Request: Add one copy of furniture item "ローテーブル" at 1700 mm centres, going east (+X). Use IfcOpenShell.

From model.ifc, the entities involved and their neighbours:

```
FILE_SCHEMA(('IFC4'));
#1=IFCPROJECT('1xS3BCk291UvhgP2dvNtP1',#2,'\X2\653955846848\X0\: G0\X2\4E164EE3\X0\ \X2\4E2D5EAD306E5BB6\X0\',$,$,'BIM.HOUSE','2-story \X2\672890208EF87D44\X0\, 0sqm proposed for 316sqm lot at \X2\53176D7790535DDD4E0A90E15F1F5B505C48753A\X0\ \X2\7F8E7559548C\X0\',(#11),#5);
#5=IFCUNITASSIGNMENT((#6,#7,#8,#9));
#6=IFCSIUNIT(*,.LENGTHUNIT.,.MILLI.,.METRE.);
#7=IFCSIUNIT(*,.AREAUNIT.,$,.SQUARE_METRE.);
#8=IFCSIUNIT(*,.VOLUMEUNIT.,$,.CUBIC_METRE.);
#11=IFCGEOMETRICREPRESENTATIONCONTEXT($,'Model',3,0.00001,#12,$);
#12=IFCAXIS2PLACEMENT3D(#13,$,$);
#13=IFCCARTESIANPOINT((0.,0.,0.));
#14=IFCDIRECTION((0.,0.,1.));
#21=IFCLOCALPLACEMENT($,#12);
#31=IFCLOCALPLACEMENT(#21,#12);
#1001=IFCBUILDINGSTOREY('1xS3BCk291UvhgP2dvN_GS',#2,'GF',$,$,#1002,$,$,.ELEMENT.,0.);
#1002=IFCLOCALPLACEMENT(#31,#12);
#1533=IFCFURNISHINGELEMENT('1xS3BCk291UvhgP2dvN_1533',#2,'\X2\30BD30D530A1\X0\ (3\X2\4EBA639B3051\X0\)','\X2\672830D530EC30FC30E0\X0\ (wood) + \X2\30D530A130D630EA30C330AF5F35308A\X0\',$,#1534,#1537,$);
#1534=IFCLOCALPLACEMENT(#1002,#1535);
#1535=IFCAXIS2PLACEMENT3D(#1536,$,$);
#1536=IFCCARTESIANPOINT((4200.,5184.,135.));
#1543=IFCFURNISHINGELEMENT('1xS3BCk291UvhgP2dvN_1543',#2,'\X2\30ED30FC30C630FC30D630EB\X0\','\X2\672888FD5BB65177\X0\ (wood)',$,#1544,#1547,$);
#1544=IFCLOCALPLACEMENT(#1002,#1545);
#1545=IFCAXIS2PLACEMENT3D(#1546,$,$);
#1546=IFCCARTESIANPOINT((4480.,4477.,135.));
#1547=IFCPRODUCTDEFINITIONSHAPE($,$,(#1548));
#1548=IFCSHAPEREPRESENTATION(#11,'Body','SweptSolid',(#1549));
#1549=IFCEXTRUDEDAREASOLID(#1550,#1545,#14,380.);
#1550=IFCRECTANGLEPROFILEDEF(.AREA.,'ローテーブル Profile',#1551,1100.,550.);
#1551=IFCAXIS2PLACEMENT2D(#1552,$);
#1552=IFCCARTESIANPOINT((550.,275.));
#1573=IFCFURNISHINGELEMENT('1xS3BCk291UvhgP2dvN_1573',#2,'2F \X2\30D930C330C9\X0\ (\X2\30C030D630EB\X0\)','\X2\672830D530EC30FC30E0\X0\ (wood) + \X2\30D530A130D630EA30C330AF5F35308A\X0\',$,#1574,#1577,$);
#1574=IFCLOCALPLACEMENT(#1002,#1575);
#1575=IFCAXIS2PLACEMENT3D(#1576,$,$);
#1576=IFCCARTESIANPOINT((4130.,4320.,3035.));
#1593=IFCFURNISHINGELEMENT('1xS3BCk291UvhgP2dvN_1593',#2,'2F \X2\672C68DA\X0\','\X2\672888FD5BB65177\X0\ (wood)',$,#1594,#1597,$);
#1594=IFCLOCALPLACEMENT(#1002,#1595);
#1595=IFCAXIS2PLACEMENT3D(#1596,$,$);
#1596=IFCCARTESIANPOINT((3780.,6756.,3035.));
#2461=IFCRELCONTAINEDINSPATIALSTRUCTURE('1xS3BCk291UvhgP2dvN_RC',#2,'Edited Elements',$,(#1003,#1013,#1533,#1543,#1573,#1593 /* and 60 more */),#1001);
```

```python
import numpy as np
import ifcopenshell
import ifcopenshell.api.geometry
import ifcopenshell.api.root
import ifcopenshell.util.element
import ifcopenshell.util.placement

model = ifcopenshell.open("model.ifc")


def reuse_history(source, copy):
    """copy_class also copies each property set's owner history, people and application; keep the originals."""
    for rel in copy.IsDefinedBy:
        if rel.is_a("IfcRelDefinesByProperties") and (history := rel.RelatingPropertyDefinition.OwnerHistory):
            rel.RelatingPropertyDefinition.OwnerHistory = source.OwnerHistory
            ifcopenshell.util.element.remove_deep2(model, history)


source = model.by_id(1543)
base = ifcopenshell.util.placement.get_local_placement(source.ObjectPlacement)
step = np.array([1.0, 0.0, 0.0]) * 1700.0

for i in range(1, 2):
    copy = ifcopenshell.api.root.copy_class(model, product=source)
    copy.Representation = ifcopenshell.util.element.copy_deep(
        model, source.Representation, exclude=["IfcGeometricRepresentationContext", "IfcRepresentationMap"]
    )
    reuse_history(source, copy)
    matrix = base.copy()
    matrix[:3, 3] += i * step
    print("added at", matrix[:3, 3].round(3) + 0.0)
    ifcopenshell.api.geometry.edit_object_placement(model, product=copy, matrix=matrix, is_si=False)

model.write("model-out.ifc")
```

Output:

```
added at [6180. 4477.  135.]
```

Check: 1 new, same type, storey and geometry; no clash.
